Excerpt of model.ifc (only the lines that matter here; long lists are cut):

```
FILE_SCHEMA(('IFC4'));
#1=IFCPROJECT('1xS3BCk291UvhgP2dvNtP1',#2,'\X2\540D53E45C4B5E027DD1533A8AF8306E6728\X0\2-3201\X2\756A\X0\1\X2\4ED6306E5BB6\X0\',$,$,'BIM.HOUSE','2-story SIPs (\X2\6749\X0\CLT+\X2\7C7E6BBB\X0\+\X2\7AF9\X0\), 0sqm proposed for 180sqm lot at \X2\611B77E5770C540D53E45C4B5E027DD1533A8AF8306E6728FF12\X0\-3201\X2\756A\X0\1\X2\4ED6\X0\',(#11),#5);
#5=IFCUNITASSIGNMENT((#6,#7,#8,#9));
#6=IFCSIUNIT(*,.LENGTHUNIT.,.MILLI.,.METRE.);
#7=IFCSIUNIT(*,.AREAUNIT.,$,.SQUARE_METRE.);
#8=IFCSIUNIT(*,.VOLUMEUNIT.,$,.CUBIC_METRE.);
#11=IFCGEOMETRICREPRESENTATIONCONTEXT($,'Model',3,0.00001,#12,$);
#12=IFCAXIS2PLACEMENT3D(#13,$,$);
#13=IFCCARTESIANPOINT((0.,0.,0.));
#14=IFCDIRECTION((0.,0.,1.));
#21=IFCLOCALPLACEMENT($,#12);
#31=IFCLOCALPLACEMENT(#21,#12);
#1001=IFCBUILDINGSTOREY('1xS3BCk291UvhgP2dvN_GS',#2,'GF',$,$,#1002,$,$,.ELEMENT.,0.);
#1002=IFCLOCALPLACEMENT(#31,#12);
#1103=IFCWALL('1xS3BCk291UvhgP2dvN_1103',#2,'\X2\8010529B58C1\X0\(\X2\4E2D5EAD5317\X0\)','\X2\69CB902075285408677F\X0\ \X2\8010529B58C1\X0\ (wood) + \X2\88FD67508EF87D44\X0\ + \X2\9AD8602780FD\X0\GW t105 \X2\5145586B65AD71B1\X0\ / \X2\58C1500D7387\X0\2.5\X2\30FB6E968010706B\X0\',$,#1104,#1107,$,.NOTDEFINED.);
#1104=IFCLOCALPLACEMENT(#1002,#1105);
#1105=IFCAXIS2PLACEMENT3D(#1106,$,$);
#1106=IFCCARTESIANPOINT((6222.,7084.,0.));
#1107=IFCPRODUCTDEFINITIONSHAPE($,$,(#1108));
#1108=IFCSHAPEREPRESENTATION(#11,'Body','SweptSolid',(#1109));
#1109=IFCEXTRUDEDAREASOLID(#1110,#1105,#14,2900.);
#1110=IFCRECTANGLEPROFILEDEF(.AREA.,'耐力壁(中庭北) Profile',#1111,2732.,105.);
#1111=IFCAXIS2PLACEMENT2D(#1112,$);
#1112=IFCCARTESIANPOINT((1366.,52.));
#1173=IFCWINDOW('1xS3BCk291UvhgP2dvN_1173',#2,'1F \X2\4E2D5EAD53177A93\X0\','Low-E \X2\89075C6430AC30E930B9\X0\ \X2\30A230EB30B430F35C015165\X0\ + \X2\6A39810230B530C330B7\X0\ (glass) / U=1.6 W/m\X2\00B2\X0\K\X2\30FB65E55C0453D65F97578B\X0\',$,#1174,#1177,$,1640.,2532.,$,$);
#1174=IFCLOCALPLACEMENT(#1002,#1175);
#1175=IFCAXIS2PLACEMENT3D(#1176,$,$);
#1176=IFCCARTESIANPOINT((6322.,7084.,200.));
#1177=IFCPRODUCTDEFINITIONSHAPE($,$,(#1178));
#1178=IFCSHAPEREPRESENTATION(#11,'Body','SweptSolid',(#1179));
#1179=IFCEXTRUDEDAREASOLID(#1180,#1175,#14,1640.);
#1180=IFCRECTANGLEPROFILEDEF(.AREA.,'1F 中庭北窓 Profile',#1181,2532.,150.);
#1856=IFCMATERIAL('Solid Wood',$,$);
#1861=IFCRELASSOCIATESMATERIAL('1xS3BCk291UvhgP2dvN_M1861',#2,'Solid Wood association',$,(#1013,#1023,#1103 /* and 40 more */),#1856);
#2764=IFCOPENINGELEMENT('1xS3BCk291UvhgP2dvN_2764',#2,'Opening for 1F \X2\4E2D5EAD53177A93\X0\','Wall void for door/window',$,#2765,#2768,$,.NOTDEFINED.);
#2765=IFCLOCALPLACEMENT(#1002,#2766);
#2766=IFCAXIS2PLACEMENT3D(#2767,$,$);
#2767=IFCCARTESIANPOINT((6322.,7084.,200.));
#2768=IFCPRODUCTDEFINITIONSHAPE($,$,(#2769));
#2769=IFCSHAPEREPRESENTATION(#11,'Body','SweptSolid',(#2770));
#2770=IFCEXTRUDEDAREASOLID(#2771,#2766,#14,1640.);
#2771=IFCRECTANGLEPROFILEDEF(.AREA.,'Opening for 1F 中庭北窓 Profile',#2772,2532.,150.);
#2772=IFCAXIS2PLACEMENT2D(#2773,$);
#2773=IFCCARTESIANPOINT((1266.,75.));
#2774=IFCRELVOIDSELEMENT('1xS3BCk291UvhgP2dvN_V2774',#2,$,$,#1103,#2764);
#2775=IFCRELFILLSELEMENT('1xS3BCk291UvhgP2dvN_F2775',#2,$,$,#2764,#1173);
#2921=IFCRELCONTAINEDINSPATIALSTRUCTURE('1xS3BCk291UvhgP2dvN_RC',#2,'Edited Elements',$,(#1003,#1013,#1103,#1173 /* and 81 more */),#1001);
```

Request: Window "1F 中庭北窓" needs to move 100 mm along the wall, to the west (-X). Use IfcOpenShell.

```python
import ifcopenshell
import ifcopenshell.api.geometry
import ifcopenshell.util.placement
import ifcopenshell.util.unit

model = ifcopenshell.open("model.ifc")
unit_scale = ifcopenshell.util.unit.calculate_unit_scale(model)

window = model.by_id(1173)
opening = window.FillsVoids[0].RelatingOpeningElement
wall = opening.VoidsElements[0].RelatingBuildingElement

wall_matrix = ifcopenshell.util.placement.get_local_placement(wall.ObjectPlacement)
shift = wall_matrix[:3, 0] * -0.1 / unit_scale
before = ifcopenshell.util.placement.get_local_placement(window.ObjectPlacement)[:3, 3].copy()

# The window is not placed relative to its opening, so move both.
for product in (opening, window):
    matrix = ifcopenshell.util.placement.get_local_placement(product.ObjectPlacement)
    matrix[:3, 3] += shift
    ifcopenshell.api.geometry.edit_object_placement(model, product=product, matrix=matrix, is_si=False)

after = ifcopenshell.util.placement.get_local_placement(window.ObjectPlacement)[:3, 3]
print("window moved by", (after - before).round(3) + 0.0)

model.write("model_rev.ifc")
```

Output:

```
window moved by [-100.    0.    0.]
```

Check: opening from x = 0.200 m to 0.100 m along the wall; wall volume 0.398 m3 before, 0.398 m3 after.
